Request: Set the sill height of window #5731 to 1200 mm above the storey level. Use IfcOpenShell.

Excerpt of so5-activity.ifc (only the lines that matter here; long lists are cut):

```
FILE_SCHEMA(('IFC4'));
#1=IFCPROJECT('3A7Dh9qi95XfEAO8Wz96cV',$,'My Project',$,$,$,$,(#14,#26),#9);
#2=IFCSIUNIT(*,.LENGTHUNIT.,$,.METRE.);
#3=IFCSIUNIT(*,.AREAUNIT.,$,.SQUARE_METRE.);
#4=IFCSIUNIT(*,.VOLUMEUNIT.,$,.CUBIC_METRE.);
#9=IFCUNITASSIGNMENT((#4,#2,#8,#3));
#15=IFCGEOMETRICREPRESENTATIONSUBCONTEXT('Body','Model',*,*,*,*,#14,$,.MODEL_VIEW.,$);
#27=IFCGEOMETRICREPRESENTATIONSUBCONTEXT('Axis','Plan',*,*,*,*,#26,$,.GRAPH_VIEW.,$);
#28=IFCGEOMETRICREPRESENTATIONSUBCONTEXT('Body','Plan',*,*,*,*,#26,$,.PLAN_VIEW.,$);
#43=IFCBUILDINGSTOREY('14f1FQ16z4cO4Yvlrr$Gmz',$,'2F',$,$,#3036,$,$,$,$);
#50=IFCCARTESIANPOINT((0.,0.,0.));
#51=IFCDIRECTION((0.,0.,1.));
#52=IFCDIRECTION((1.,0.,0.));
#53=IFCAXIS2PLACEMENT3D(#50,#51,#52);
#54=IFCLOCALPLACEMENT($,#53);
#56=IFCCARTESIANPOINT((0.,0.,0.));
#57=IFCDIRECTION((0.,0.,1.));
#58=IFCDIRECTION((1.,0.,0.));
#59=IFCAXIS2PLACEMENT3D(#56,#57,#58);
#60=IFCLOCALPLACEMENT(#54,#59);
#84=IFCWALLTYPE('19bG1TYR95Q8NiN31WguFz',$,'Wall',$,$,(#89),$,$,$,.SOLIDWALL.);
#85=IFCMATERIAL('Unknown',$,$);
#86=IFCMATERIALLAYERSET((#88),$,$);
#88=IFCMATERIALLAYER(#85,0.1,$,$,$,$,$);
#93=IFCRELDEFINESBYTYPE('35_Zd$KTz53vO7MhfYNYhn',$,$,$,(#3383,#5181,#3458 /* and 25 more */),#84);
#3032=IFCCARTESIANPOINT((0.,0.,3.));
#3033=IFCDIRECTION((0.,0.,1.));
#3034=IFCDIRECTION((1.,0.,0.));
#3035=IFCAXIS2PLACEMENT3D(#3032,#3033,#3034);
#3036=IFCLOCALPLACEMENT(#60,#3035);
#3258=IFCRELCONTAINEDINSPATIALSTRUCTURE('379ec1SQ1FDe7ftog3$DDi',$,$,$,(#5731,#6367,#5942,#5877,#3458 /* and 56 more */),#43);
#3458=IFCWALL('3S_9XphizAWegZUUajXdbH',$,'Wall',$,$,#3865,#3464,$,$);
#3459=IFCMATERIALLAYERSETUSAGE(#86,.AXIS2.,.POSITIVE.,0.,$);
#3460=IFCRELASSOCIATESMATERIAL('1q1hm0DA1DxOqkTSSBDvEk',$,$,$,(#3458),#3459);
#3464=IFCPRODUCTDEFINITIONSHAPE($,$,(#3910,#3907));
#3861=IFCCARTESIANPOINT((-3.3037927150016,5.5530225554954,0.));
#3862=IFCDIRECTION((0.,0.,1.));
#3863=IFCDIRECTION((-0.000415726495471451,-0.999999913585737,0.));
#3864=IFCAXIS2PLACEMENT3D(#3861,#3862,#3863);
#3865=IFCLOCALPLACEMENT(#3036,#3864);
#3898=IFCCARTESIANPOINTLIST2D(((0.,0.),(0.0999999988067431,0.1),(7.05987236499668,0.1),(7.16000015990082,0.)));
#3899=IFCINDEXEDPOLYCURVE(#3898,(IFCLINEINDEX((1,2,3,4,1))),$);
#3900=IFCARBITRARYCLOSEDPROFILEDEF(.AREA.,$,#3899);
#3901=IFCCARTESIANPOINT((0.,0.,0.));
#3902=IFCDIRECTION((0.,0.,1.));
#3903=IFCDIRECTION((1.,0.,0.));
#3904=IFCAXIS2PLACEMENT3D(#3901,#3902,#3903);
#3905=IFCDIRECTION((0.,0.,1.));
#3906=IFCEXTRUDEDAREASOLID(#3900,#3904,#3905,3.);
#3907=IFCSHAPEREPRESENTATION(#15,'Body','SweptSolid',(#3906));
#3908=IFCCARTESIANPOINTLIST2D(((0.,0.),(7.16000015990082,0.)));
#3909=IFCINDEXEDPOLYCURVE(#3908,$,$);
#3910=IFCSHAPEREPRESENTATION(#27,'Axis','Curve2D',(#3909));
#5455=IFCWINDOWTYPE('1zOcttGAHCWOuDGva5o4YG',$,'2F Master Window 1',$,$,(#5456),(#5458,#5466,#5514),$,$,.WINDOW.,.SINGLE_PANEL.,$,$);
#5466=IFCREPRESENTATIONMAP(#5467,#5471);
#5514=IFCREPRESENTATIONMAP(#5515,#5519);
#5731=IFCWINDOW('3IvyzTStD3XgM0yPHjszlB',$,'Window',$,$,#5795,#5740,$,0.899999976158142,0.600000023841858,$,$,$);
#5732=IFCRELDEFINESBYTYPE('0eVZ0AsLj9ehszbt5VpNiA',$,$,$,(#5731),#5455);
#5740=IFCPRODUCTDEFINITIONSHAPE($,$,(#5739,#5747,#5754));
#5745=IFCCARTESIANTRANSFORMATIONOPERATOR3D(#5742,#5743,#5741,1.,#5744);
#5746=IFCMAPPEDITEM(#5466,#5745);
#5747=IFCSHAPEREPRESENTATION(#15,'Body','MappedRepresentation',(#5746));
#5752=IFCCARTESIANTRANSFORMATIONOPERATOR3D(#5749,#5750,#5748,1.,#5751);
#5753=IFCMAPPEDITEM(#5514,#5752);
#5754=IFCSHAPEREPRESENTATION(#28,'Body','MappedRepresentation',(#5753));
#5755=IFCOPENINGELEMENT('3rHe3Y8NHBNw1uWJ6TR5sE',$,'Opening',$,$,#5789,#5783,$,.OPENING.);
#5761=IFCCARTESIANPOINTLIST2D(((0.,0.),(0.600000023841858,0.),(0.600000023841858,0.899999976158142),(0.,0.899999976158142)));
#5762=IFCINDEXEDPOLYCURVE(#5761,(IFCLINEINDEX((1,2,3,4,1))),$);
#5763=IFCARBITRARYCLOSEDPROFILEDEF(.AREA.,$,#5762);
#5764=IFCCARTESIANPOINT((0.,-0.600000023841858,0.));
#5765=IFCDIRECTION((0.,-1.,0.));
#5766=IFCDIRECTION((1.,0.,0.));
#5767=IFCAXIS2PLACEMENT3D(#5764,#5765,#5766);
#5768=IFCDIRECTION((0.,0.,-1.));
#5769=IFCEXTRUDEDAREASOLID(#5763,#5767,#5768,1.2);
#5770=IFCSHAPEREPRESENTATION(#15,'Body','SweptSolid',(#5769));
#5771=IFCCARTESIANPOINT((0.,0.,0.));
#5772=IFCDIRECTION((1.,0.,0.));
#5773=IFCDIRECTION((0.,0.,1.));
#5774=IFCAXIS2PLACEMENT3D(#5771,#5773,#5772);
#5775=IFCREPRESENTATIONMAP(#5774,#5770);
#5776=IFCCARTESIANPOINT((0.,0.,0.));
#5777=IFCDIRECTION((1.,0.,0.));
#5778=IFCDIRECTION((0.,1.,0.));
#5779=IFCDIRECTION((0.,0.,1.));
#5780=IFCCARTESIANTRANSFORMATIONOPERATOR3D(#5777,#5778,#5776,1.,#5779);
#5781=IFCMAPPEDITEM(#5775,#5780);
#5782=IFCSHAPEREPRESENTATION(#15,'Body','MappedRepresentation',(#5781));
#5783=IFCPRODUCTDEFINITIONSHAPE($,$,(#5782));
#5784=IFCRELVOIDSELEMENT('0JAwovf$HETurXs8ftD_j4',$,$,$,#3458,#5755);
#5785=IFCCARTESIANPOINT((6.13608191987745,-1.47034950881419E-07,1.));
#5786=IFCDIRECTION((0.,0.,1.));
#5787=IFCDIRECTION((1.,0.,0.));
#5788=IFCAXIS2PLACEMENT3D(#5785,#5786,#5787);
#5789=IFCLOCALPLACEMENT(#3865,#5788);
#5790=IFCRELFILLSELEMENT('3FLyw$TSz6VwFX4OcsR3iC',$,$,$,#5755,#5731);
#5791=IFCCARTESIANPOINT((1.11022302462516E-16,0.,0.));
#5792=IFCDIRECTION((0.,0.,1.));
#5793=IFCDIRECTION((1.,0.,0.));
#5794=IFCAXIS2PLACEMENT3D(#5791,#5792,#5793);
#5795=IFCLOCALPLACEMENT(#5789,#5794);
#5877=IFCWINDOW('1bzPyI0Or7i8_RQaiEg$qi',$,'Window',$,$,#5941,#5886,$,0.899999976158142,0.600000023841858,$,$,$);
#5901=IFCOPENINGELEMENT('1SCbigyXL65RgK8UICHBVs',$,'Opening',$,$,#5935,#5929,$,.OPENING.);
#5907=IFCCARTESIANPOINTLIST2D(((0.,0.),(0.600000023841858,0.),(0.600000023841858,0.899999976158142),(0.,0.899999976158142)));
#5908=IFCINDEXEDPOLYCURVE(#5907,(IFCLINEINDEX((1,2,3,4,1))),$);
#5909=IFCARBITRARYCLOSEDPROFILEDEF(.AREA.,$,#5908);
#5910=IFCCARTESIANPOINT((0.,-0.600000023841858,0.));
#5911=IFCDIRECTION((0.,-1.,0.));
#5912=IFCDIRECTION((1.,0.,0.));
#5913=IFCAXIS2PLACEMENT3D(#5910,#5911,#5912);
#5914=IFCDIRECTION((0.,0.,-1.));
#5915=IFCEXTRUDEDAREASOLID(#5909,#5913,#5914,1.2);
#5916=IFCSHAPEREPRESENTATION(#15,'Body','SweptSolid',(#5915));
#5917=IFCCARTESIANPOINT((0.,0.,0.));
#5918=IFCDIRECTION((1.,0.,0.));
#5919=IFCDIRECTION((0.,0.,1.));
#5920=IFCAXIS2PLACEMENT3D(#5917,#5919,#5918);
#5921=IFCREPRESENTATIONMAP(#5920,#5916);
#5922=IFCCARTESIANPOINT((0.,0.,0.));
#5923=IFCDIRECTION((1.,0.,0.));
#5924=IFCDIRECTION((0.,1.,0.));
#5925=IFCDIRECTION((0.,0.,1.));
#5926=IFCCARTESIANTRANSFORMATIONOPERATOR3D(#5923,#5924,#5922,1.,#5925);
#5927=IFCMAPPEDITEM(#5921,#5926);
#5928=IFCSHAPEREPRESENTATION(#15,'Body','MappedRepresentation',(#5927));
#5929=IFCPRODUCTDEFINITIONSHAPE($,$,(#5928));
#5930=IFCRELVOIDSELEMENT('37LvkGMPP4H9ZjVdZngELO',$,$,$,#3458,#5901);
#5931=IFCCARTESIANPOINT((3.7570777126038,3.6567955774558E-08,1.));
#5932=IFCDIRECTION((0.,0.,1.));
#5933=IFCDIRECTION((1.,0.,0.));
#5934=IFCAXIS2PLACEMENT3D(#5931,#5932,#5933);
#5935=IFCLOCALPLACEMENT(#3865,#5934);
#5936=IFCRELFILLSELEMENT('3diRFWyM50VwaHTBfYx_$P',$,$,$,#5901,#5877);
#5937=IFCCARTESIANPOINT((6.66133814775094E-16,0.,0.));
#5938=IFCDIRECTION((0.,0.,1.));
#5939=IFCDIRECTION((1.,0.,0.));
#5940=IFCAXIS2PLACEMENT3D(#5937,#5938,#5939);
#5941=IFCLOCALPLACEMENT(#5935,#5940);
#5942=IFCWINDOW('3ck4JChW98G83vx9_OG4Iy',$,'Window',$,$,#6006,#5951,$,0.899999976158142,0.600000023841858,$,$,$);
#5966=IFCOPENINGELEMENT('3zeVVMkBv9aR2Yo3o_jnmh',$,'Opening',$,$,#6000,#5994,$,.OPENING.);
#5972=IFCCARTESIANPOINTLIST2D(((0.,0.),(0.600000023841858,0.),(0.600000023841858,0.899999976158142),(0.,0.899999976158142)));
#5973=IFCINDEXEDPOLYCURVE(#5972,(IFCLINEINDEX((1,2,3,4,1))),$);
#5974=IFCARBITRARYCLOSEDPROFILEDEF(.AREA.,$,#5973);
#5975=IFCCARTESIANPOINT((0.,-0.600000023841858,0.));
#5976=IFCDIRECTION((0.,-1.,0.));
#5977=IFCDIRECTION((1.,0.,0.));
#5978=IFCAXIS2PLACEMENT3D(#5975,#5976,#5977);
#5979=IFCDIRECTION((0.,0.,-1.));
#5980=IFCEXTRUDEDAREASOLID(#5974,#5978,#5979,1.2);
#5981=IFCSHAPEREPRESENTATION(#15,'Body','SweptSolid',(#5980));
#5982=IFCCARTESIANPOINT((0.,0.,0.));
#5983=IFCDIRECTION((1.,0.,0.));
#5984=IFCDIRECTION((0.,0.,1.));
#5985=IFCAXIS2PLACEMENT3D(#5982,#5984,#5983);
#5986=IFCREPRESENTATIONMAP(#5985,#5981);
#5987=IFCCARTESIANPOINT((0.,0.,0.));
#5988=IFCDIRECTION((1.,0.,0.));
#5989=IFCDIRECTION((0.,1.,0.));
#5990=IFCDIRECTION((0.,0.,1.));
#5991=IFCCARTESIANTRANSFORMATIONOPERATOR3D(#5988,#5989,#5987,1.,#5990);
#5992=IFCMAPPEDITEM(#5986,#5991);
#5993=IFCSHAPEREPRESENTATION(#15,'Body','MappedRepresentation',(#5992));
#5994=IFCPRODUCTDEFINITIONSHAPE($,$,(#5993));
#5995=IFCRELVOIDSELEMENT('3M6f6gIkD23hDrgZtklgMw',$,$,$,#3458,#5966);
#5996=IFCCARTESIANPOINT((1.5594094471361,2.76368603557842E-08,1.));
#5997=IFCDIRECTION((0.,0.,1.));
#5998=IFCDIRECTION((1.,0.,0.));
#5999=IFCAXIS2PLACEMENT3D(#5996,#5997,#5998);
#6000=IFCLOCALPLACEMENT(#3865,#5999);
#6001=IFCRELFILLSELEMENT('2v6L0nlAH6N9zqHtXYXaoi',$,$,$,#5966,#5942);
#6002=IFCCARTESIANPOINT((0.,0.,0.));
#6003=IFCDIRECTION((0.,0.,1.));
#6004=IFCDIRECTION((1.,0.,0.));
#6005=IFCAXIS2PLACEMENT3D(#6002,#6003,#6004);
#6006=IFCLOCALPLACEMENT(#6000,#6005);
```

```python
import numpy as np
import ifcopenshell
import ifcopenshell.api.geometry
import ifcopenshell.geom
import ifcopenshell.util.element
import ifcopenshell.util.placement
import ifcopenshell.util.shape
import ifcopenshell.util.unit

model = ifcopenshell.open("so5-activity.ifc")
unit_scale = ifcopenshell.util.unit.calculate_unit_scale(model)

window = model.by_guid("3IvyzTStD3XgM0yPHjszlB")
opening = window.FillsVoids[0].RelatingOpeningElement
storey = ifcopenshell.util.element.get_container(window, ifc_class="IfcBuildingStorey")
level = ifcopenshell.util.placement.get_local_placement(storey.ObjectPlacement)[2, 3]

# The opening's origin need not be at the sill, so measure its lowest point.
shape = ifcopenshell.geom.create_shape(ifcopenshell.geom.settings(), opening)
bottom = ifcopenshell.util.shape.get_shape_bottom_elevation(shape, shape.geometry) / unit_scale
dz = level + 1.2 - bottom

shift = np.array([0.0, 0.0, dz])
# The window is placed relative to its opening, so it follows when the opening moves.
matrix = ifcopenshell.util.placement.get_local_placement(opening.ObjectPlacement)
matrix[:3, 3] += shift
ifcopenshell.api.geometry.edit_object_placement(
    model, product=opening, matrix=matrix, is_si=False, should_transform_children=True
)

print(f"moved by {dz * unit_scale:+.3f} m")

model.write("so5-activity_rev.ifc")
```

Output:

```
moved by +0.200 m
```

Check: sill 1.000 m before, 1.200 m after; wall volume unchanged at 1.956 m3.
